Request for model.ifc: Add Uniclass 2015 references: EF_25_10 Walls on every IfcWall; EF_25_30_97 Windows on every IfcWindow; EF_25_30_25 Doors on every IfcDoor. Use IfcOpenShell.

First a look at what the model holds.

```python
import ifcopenshell

model = ifcopenshell.open("model.ifc")
print(model.schema)
print("classifications:", [c.Name for c in model.by_type("IfcClassification")])
for ifc_class in ("IfcDoor", "IfcRoof", "IfcStair", "IfcWall", "IfcWindow"):
    print(ifc_class, len(model.by_type(ifc_class)))
```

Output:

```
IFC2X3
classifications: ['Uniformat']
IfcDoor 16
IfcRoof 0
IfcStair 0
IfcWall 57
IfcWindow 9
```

```python
import ifcopenshell
import ifcopenshell.api.classification

model = ifcopenshell.open("model.ifc")

# IFC2X3 requires Source and Edition and has no link from the project to the system.
system = model.create_entity("IfcClassification", Source="NBS", Edition="2015", Name="Uniclass 2015")

codes = {
    "IfcWall": ("EF_25_10", "Walls"),
    "IfcWindow": ("EF_25_30_97", "Windows"),
    "IfcDoor": ("EF_25_30_25", "Doors"),
}
for ifc_class, (code, name) in codes.items():
    products = model.by_type(ifc_class)
    ifcopenshell.api.classification.add_reference(
        model, products=products, classification=system, identification=code, name=name
    )
    print(code, len(products))

model.write("model_v2.ifc")
```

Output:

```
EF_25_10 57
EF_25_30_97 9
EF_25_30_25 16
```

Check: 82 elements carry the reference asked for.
